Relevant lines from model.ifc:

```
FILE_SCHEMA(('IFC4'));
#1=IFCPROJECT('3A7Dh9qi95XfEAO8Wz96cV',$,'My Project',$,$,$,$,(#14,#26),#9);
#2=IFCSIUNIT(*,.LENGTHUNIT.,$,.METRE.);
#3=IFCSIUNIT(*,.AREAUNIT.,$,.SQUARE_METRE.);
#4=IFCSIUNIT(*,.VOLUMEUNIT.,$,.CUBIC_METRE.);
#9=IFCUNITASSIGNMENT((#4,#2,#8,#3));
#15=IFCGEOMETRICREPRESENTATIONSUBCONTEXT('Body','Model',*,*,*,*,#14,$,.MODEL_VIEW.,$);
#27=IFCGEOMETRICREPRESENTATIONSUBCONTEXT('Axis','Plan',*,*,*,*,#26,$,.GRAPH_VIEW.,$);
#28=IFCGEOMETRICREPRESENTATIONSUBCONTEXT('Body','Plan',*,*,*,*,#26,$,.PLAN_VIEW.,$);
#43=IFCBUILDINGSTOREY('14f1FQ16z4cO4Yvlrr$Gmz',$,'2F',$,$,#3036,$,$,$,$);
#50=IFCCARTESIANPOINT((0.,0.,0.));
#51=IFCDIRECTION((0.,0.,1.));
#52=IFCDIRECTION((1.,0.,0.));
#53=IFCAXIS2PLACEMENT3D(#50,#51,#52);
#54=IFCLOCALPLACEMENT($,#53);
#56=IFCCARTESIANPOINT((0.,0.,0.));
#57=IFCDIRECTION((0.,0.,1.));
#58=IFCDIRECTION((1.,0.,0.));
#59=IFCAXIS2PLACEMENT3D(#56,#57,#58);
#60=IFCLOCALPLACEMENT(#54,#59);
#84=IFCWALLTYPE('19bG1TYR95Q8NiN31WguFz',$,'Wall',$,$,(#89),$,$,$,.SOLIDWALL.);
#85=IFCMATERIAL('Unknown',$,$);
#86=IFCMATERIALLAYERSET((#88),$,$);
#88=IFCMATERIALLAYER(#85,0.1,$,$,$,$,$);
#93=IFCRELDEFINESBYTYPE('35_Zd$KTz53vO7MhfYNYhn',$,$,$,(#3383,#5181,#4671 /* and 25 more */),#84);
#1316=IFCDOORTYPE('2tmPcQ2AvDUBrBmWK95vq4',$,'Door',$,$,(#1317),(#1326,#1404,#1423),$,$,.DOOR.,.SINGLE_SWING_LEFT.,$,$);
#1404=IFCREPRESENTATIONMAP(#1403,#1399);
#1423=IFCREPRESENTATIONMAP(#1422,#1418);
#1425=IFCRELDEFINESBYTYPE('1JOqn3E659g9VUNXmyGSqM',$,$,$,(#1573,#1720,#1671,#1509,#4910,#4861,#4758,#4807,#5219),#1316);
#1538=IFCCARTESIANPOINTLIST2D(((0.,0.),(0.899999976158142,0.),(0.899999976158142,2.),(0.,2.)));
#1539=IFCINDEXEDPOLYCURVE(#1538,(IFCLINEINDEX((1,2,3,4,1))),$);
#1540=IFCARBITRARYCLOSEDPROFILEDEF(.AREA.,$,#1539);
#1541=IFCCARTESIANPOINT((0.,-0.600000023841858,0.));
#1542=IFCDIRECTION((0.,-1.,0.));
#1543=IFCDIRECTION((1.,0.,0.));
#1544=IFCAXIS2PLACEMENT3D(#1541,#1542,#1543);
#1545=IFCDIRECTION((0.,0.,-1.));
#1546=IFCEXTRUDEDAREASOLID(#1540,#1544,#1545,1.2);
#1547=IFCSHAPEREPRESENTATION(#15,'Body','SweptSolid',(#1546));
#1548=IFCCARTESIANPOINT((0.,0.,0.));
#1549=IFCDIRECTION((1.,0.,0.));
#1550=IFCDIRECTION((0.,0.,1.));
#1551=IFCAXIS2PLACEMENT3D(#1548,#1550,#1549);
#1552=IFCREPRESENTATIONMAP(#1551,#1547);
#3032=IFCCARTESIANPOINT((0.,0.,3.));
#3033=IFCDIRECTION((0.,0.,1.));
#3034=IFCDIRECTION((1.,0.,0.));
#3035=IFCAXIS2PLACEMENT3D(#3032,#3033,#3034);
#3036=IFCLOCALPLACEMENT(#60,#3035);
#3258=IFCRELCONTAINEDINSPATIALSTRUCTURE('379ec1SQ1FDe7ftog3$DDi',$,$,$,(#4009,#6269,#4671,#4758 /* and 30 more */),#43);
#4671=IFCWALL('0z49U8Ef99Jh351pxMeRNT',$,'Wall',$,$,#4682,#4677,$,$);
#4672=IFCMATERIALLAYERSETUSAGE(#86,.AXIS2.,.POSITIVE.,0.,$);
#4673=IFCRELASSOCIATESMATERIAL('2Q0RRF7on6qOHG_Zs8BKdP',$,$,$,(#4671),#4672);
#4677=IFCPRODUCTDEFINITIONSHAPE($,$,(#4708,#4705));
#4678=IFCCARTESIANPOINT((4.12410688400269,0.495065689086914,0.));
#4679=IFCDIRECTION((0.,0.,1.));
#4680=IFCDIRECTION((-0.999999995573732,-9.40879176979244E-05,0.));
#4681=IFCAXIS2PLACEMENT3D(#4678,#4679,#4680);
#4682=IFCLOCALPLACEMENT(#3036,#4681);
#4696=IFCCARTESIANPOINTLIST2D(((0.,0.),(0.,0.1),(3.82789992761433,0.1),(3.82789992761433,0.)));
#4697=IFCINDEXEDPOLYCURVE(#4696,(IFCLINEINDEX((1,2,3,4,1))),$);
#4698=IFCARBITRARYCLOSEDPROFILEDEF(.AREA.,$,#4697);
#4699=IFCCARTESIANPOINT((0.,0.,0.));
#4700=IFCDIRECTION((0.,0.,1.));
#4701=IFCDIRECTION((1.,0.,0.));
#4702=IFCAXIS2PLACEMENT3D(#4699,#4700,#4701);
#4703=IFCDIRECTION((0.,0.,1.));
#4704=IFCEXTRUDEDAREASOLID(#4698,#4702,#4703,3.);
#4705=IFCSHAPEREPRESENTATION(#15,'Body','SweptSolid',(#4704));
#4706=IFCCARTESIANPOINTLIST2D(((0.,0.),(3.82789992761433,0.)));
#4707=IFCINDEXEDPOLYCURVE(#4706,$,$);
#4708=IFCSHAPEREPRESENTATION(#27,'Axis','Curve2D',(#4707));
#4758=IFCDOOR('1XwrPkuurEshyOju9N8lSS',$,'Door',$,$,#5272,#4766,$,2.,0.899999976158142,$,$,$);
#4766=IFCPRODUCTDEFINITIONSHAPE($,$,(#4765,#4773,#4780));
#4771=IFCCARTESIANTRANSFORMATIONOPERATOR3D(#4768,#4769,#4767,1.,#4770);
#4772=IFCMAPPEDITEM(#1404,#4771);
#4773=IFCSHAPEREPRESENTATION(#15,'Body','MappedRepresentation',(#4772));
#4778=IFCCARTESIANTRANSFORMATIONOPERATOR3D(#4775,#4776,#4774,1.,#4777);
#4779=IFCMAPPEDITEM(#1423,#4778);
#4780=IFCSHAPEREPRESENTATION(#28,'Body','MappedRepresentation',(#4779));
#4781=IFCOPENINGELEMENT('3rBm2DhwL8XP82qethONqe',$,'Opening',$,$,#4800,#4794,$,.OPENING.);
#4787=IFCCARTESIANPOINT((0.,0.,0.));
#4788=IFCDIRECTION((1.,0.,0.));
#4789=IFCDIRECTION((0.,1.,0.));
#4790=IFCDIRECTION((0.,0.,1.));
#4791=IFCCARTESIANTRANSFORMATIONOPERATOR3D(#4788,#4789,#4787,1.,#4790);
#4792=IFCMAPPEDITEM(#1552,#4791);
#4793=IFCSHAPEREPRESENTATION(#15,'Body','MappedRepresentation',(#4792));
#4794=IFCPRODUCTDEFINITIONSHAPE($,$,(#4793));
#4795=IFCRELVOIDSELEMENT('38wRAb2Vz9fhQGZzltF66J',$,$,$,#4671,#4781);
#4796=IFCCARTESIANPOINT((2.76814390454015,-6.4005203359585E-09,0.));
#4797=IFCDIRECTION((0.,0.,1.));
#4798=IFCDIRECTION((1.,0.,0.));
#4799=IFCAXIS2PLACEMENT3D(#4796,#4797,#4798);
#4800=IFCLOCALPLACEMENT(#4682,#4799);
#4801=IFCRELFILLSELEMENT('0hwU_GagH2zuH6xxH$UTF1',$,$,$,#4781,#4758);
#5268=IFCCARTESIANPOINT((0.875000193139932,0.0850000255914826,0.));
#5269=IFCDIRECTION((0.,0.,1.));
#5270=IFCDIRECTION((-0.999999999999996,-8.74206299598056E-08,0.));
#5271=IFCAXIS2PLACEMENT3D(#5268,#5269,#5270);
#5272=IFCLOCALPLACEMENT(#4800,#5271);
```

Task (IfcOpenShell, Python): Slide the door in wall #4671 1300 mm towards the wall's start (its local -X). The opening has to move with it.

```python
import ifcopenshell
import ifcopenshell.api.geometry
import ifcopenshell.util.placement
import ifcopenshell.util.unit

model = ifcopenshell.open("model.ifc")
unit_scale = ifcopenshell.util.unit.calculate_unit_scale(model)

door = model.by_guid("1XwrPkuurEshyOju9N8lSS")
opening = door.FillsVoids[0].RelatingOpeningElement
wall = opening.VoidsElements[0].RelatingBuildingElement

wall_matrix = ifcopenshell.util.placement.get_local_placement(wall.ObjectPlacement)
shift = wall_matrix[:3, 0] * -1.3 / unit_scale
before = ifcopenshell.util.placement.get_local_placement(door.ObjectPlacement)[:3, 3].copy()

# The door is placed relative to its opening, so it follows when the opening moves.
matrix = ifcopenshell.util.placement.get_local_placement(opening.ObjectPlacement)
matrix[:3, 3] += shift
ifcopenshell.api.geometry.edit_object_placement(
    model, product=opening, matrix=matrix, is_si=False, should_transform_children=True
)

after = ifcopenshell.util.placement.get_local_placement(door.ObjectPlacement)[:3, 3]
print("door moved by", (after - before).round(3) + 0.0)

model.write("model_v2.ifc")
```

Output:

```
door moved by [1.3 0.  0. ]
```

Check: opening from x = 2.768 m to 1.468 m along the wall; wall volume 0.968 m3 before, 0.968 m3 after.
